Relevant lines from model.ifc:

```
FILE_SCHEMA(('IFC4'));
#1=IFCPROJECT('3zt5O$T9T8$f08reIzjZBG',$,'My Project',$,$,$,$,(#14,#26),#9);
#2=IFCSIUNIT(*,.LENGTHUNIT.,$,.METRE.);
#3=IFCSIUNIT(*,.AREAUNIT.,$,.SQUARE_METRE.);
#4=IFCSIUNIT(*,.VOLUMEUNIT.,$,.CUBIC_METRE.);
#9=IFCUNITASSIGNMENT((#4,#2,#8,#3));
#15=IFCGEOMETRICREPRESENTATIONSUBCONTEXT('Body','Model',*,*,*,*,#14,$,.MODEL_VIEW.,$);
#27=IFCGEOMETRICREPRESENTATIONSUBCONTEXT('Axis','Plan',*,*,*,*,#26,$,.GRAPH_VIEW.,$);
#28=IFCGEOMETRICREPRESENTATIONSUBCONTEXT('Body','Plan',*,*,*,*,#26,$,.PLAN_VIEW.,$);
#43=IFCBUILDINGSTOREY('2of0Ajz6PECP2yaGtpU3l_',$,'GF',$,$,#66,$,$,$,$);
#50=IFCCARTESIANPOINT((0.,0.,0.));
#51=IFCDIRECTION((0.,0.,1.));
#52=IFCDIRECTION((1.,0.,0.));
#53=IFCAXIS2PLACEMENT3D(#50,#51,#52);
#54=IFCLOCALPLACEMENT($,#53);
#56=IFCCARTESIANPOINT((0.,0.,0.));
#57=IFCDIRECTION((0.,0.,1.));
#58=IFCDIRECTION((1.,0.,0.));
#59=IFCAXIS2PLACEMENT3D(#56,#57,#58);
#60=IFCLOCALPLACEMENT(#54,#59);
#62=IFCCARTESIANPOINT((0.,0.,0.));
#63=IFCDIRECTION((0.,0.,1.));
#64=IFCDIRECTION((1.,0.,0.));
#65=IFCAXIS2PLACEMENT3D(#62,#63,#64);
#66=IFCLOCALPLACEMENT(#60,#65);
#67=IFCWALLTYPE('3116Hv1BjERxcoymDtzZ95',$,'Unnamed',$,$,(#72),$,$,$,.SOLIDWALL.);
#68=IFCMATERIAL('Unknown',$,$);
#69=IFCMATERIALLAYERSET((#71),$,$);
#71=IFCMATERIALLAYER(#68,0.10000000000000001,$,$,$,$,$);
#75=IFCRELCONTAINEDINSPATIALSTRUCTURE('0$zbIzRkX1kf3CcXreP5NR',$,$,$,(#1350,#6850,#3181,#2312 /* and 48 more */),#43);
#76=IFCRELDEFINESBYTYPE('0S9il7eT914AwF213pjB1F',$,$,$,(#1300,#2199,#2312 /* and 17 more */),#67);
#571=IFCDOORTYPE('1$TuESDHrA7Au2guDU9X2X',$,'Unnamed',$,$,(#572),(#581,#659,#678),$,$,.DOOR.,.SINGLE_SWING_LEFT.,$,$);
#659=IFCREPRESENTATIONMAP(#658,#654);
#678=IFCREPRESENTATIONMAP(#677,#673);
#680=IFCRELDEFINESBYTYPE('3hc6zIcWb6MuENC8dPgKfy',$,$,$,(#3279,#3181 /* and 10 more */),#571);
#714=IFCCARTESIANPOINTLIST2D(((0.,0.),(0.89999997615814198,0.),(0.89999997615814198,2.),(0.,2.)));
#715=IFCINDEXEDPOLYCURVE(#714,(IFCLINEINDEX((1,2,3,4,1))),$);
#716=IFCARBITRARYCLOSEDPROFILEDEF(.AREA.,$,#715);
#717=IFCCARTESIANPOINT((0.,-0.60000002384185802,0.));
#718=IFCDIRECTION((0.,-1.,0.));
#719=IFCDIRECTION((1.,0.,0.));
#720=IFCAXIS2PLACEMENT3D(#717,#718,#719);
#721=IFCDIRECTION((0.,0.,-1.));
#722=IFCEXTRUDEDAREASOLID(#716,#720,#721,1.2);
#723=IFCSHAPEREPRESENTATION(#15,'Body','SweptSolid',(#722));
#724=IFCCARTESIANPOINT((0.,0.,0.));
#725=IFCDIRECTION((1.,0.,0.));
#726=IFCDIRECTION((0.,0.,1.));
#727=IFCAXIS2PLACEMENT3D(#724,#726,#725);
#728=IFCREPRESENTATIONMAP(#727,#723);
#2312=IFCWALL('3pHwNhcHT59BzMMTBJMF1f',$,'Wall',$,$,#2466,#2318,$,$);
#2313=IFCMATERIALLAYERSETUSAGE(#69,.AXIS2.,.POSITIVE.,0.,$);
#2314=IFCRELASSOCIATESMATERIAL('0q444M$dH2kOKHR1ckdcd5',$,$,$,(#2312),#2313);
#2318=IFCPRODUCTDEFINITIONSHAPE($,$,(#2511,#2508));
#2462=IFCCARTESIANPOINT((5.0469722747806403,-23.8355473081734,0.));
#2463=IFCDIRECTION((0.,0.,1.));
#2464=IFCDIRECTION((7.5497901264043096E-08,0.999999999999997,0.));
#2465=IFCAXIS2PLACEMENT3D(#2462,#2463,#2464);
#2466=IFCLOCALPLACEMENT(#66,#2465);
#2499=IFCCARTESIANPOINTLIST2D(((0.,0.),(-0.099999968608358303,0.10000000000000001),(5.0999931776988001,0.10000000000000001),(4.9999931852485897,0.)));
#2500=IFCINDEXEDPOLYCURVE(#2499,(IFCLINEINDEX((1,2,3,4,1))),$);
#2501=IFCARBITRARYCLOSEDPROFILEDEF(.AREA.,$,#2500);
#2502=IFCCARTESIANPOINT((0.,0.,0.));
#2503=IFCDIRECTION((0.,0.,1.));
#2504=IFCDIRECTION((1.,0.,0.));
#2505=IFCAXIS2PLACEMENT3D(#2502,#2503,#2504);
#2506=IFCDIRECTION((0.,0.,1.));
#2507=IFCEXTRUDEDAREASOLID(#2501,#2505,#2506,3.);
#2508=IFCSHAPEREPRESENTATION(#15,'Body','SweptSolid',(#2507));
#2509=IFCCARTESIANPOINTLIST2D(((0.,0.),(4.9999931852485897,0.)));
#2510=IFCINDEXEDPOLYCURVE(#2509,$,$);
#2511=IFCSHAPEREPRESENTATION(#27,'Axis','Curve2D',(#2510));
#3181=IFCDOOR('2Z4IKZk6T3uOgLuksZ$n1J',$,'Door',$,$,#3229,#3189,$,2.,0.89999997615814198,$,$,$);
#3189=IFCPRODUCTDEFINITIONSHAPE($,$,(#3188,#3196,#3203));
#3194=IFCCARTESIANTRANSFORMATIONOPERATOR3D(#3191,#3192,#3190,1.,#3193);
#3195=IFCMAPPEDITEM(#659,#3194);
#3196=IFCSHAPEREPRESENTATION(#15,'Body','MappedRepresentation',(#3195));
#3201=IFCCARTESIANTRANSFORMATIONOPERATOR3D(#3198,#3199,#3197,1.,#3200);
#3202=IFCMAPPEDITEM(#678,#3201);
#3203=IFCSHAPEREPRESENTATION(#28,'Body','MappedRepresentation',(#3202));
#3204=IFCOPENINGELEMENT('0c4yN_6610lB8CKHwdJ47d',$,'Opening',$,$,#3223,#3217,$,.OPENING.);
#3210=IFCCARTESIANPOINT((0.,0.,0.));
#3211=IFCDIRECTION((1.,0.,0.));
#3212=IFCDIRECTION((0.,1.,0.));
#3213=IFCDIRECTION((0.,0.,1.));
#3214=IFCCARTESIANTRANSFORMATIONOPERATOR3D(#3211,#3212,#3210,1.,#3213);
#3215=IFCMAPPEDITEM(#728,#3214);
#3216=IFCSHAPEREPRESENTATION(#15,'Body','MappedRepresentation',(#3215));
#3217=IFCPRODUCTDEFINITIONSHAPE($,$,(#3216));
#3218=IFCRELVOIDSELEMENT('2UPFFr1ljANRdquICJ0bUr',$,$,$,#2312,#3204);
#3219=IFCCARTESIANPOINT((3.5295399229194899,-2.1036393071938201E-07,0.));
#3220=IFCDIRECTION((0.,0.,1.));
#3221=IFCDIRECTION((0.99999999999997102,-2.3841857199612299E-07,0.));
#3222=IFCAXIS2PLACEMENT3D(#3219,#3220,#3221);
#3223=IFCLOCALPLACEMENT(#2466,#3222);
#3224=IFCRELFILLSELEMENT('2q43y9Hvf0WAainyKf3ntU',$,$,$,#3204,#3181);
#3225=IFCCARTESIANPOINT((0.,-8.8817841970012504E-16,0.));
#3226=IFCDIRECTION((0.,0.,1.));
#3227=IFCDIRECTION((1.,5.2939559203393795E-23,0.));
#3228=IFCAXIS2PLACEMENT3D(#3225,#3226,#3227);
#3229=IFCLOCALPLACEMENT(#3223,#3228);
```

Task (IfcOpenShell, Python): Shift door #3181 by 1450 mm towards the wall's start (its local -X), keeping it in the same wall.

```python
import ifcopenshell
import ifcopenshell.api.geometry
import ifcopenshell.util.placement
import ifcopenshell.util.unit

model = ifcopenshell.open("model.ifc")
unit_scale = ifcopenshell.util.unit.calculate_unit_scale(model)

door = model.by_guid("2Z4IKZk6T3uOgLuksZ$n1J")
opening = door.FillsVoids[0].RelatingOpeningElement
wall = opening.VoidsElements[0].RelatingBuildingElement

wall_matrix = ifcopenshell.util.placement.get_local_placement(wall.ObjectPlacement)
shift = wall_matrix[:3, 0] * -1.45 / unit_scale
before = ifcopenshell.util.placement.get_local_placement(door.ObjectPlacement)[:3, 3].copy()

# The door is placed relative to its opening, so it follows when the opening moves.
matrix = ifcopenshell.util.placement.get_local_placement(opening.ObjectPlacement)
matrix[:3, 3] += shift
ifcopenshell.api.geometry.edit_object_placement(
    model, product=opening, matrix=matrix, is_si=False, should_transform_children=True
)

after = ifcopenshell.util.placement.get_local_placement(door.ObjectPlacement)[:3, 3]
print("door moved by", (after - before).round(3) + 0.0)

model.write("model_updated.ifc")
```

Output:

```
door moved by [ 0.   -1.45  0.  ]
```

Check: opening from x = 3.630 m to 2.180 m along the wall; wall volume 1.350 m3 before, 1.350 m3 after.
